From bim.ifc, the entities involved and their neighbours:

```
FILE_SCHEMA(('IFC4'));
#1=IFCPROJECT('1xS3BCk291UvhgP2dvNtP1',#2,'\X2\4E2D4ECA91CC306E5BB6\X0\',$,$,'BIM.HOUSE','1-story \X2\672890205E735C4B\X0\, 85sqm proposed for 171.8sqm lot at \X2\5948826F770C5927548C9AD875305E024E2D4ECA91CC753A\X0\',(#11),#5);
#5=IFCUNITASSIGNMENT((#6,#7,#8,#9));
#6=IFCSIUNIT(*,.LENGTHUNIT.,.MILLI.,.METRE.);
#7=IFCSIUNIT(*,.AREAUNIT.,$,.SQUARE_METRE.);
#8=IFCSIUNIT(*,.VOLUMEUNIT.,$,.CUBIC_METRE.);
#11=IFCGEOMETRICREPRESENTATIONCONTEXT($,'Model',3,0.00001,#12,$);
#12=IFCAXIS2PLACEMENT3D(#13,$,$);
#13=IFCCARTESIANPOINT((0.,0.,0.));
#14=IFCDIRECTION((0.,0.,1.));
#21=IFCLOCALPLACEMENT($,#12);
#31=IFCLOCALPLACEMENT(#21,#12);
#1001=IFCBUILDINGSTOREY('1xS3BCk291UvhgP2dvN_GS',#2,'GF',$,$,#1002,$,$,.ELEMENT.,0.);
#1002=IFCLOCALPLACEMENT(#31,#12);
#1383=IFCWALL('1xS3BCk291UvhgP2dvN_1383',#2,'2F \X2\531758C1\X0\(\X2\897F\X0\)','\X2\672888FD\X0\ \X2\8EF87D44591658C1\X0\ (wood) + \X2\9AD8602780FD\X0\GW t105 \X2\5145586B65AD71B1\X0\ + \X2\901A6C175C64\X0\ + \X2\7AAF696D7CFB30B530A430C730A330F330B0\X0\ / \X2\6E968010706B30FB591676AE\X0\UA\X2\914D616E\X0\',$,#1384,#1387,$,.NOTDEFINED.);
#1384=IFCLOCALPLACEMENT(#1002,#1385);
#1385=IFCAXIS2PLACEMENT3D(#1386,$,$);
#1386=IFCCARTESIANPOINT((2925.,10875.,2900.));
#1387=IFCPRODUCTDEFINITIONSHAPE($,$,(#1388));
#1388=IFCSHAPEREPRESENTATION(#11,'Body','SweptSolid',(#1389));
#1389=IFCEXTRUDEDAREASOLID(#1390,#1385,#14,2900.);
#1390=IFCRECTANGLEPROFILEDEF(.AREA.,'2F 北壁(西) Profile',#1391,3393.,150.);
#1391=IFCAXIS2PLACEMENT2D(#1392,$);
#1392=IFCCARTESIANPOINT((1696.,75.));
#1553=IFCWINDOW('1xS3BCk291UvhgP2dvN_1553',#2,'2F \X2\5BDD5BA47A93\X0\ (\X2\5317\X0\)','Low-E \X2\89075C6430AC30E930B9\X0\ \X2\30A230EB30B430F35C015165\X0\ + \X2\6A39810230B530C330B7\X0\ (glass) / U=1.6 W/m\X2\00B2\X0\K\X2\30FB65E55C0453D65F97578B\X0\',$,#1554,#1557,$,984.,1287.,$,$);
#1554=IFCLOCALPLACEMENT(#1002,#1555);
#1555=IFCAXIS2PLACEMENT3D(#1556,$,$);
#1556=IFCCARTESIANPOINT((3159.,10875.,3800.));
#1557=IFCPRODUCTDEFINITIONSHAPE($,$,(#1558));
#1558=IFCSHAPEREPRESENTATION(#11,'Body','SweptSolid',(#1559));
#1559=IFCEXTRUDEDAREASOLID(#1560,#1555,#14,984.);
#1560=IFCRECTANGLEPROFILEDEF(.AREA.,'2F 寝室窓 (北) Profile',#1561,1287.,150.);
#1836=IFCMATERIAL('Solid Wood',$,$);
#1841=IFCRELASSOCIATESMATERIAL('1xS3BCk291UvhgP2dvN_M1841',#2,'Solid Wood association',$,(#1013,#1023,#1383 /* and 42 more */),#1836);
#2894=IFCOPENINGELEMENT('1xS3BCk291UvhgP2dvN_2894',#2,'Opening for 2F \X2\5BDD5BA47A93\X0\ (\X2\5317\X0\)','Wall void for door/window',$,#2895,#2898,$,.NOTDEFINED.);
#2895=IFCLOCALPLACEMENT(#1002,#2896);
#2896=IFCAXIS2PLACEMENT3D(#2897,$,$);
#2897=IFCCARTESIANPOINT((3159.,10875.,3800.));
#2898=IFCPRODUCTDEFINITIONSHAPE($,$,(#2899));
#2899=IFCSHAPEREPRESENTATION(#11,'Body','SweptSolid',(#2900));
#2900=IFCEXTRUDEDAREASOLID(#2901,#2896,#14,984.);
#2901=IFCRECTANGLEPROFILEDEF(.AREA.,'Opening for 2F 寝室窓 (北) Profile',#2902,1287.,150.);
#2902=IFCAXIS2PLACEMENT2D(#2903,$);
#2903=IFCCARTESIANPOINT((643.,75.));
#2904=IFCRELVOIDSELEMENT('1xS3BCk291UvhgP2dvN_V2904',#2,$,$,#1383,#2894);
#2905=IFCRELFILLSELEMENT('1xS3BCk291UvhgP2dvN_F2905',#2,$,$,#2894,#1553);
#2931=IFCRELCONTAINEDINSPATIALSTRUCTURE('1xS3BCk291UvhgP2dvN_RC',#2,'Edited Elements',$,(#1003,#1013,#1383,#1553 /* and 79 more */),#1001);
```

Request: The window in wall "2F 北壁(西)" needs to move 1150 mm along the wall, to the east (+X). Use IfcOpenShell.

```python
import ifcopenshell
import ifcopenshell.api.geometry
import ifcopenshell.util.placement
import ifcopenshell.util.unit

model = ifcopenshell.open("bim.ifc")
unit_scale = ifcopenshell.util.unit.calculate_unit_scale(model)

window = model.by_guid("1xS3BCk291UvhgP2dvN_1553")
opening = window.FillsVoids[0].RelatingOpeningElement
wall = opening.VoidsElements[0].RelatingBuildingElement

wall_matrix = ifcopenshell.util.placement.get_local_placement(wall.ObjectPlacement)
shift = wall_matrix[:3, 0] * 1.15 / unit_scale
before = ifcopenshell.util.placement.get_local_placement(window.ObjectPlacement)[:3, 3].copy()

# The window is not placed relative to its opening, so move both.
for product in (opening, window):
    matrix = ifcopenshell.util.placement.get_local_placement(product.ObjectPlacement)
    matrix[:3, 3] += shift
    ifcopenshell.api.geometry.edit_object_placement(model, product=product, matrix=matrix, is_si=False)

after = ifcopenshell.util.placement.get_local_placement(window.ObjectPlacement)[:3, 3]
print("window moved by", (after - before).round(3) + 0.0)

model.write("bim_rev.ifc")
```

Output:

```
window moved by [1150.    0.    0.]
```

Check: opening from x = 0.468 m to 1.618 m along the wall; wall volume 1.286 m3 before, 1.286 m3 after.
